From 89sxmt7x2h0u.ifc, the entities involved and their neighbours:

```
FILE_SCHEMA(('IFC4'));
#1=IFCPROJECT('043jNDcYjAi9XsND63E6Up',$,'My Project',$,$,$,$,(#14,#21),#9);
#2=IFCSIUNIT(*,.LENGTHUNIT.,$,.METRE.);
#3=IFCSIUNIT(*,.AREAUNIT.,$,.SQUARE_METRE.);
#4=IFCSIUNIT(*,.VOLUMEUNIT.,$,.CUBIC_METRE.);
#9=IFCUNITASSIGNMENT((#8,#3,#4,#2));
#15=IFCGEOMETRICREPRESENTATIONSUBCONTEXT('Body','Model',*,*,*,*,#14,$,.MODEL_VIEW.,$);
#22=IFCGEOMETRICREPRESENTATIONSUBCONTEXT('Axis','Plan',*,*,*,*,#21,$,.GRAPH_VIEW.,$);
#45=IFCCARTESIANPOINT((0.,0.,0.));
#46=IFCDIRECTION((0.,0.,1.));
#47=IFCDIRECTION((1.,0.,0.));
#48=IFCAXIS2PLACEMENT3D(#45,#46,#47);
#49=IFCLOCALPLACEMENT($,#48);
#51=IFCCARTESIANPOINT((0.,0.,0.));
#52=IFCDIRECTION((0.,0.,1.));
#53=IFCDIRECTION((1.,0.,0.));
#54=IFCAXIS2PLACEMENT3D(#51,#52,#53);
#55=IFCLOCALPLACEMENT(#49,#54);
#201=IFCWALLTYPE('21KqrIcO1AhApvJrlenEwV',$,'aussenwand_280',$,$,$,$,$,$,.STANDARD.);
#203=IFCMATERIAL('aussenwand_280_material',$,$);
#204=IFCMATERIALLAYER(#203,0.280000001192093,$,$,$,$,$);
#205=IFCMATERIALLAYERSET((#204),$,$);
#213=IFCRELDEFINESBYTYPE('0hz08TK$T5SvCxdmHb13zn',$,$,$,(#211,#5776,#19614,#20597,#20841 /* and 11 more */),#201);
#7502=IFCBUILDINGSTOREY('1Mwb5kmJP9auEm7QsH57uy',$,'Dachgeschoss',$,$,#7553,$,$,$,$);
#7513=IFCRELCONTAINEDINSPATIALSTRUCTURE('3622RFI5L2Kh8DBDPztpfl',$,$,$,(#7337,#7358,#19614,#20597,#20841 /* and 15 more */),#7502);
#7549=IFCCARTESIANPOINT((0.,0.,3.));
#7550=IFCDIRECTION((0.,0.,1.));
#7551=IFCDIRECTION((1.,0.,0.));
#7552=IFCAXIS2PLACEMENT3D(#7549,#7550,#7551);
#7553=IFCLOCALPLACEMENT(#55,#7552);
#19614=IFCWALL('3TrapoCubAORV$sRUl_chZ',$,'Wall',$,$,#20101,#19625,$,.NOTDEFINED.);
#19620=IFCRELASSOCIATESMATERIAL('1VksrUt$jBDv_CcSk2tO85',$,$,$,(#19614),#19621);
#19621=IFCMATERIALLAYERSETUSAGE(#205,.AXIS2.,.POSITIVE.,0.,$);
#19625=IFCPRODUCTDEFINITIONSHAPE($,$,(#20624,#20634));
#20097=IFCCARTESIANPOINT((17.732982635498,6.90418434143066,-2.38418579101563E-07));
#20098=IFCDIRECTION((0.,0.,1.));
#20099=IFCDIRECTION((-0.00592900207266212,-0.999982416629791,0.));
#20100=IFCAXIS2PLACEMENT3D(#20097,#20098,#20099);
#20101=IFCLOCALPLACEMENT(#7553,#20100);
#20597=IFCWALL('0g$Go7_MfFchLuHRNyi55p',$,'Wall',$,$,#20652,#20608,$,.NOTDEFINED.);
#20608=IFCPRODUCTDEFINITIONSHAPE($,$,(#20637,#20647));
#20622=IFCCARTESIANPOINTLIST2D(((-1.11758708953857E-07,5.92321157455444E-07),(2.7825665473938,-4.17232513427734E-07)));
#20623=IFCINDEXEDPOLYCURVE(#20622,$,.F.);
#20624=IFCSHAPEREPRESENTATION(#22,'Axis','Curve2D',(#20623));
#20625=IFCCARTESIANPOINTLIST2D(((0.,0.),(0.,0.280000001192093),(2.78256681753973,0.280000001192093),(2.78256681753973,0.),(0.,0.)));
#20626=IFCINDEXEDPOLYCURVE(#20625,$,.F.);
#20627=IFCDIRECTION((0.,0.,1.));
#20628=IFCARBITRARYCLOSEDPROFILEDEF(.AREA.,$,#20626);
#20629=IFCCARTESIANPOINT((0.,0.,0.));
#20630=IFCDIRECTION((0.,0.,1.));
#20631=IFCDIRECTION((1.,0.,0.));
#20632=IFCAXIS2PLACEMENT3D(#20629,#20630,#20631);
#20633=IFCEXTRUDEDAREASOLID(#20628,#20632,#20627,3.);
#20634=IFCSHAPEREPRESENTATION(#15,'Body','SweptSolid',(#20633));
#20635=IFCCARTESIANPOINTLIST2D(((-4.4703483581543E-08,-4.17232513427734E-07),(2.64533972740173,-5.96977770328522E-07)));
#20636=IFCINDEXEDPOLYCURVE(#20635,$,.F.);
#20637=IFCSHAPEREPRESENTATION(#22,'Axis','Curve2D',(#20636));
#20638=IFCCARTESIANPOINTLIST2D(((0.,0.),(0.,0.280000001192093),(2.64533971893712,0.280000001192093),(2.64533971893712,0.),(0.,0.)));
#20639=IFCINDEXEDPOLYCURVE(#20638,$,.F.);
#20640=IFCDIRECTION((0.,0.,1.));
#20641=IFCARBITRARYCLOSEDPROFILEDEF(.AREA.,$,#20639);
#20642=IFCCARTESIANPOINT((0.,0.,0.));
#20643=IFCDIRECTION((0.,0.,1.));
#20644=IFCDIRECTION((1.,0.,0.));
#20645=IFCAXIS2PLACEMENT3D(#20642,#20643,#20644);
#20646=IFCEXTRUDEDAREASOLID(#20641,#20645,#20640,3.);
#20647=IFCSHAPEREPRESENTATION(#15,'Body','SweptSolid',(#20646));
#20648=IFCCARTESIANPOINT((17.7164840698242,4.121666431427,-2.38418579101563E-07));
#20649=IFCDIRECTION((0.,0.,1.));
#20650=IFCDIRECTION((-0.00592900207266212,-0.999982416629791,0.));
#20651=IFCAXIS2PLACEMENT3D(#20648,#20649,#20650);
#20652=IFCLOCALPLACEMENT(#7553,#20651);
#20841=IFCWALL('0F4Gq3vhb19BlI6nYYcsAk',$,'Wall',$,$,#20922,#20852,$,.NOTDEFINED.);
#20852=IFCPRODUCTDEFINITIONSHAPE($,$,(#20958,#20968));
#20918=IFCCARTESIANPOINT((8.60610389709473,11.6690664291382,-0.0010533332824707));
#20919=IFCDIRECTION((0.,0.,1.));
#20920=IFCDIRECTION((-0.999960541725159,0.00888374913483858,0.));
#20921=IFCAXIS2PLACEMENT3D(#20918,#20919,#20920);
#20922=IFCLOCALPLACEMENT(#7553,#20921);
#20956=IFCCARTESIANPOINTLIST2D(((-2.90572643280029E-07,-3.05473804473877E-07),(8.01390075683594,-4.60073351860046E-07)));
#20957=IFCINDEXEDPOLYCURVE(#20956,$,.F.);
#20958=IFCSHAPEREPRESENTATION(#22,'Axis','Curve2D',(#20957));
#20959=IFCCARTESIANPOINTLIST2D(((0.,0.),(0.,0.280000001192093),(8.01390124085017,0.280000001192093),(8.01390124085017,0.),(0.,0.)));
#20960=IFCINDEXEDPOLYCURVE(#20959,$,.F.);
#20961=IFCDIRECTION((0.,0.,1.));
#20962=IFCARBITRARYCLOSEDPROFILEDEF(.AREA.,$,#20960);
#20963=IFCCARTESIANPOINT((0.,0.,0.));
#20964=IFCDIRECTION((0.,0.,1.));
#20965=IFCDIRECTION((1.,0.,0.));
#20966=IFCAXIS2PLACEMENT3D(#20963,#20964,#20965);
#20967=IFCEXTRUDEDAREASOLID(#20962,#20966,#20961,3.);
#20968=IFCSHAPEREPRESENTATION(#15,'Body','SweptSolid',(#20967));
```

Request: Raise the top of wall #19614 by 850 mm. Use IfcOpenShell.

```python
import ifcopenshell
import ifcopenshell.geom
import ifcopenshell.util.representation
import ifcopenshell.util.shape
import ifcopenshell.util.unit

model = ifcopenshell.open("89sxmt7x2h0u.ifc")
unit_scale = ifcopenshell.util.unit.calculate_unit_scale(model)
settings = ifcopenshell.geom.settings()


def volume(element):
    """Net volume in cubic metres, openings subtracted."""
    shape = ifcopenshell.geom.create_shape(settings, element)
    return ifcopenshell.util.shape.get_volume(shape.geometry)


wall = model.by_id(19614)
before = volume(wall)

body = ifcopenshell.util.representation.get_representation(wall, "Model", "Body")
solid = body.Items[0]
old_height = solid.Depth
solid.Depth += 0.85 / unit_scale
after = volume(wall)

print(f"height {old_height:g} -> {solid.Depth:g}, volume {before:.3f} -> {after:.3f} m3")

model.write("89sxmt7x2h0u-out.ifc")
```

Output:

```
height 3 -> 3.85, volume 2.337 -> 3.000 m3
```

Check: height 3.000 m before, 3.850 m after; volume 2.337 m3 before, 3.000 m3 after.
